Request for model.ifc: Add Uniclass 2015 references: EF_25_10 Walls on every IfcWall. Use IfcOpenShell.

First a look at what the model holds.

```python
import ifcopenshell

model = ifcopenshell.open("model.ifc")
print(model.schema)
print("classifications:", [c.Name for c in model.by_type("IfcClassification")])
for ifc_class in ("IfcDoor", "IfcRoof", "IfcStair", "IfcWall", "IfcWindow"):
    print(ifc_class, len(model.by_type(ifc_class)))
```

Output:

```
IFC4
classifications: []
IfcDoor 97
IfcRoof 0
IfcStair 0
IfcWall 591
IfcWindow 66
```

```python
import ifcopenshell
import ifcopenshell.api.classification

model = ifcopenshell.open("model.ifc")

system = ifcopenshell.api.classification.add_classification(model, classification="Uniclass 2015")

codes = {
    "IfcWall": ("EF_25_10", "Walls"),
}
for ifc_class, (code, name) in codes.items():
    products = model.by_type(ifc_class)
    ifcopenshell.api.classification.add_reference(
        model, products=products, classification=system, identification=code, name=name
    )
    print(code, len(products))

model.write("model-out.ifc")
```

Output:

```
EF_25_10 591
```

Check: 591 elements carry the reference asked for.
